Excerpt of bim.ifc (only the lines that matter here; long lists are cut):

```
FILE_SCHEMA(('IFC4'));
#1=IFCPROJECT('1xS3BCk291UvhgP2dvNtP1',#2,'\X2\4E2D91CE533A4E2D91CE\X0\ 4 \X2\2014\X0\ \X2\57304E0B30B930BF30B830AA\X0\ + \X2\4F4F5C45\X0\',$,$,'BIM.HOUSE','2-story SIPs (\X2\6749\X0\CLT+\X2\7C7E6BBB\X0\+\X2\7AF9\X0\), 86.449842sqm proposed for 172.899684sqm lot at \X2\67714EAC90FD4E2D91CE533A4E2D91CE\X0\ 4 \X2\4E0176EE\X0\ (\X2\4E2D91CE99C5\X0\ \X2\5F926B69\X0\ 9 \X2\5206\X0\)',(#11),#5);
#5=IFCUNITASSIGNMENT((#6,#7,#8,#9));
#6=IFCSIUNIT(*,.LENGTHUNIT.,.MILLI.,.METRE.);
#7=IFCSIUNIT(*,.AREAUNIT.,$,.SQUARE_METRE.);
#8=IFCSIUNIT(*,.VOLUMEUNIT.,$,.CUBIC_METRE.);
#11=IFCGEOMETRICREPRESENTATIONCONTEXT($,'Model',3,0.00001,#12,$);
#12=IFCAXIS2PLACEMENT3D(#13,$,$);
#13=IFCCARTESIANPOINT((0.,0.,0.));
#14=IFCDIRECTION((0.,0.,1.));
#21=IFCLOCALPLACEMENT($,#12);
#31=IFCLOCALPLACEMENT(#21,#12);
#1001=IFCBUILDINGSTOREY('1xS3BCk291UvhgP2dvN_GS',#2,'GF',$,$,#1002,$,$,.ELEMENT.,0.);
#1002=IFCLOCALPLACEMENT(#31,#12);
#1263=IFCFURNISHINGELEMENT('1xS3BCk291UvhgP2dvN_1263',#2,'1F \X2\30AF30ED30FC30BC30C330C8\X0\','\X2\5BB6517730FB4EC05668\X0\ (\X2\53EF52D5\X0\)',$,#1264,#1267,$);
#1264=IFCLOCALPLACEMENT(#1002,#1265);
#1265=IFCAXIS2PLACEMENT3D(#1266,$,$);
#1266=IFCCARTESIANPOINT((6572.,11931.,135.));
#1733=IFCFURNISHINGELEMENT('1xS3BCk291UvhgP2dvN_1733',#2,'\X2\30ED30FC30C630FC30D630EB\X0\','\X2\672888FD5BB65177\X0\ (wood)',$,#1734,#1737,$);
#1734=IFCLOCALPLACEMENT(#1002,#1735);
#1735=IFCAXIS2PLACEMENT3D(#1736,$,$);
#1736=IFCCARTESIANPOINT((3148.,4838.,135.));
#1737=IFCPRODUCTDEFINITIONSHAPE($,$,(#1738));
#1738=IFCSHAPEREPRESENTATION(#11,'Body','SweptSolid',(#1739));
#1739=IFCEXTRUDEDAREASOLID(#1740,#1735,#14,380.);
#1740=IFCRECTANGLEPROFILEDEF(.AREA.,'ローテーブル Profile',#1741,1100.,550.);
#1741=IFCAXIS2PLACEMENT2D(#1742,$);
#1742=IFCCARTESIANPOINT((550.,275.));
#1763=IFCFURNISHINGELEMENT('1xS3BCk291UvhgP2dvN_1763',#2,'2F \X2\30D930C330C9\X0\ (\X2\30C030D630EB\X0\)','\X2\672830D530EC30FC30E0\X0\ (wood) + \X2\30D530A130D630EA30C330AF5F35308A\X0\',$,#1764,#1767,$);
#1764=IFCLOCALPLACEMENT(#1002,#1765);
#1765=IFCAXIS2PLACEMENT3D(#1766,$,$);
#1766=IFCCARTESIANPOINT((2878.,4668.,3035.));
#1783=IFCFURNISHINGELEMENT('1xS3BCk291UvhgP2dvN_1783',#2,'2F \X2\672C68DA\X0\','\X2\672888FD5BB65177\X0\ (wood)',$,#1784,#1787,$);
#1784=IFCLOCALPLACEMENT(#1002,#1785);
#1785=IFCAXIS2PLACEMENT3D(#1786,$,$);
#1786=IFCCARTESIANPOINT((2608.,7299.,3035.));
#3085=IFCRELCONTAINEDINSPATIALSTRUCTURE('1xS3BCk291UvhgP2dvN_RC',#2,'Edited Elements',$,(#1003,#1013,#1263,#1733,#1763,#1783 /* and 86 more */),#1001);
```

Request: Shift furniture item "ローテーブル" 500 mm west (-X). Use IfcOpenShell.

```python
import ifcopenshell
import ifcopenshell.api.geometry
import ifcopenshell.util.placement

model = ifcopenshell.open("bim.ifc")

item = model.by_guid("1xS3BCk291UvhgP2dvN_1733")
matrix = ifcopenshell.util.placement.get_local_placement(item.ObjectPlacement)
matrix[0, 3] -= 500.0
ifcopenshell.api.geometry.edit_object_placement(model, product=item, matrix=matrix, is_si=False)

print(ifcopenshell.util.placement.get_local_placement(item.ObjectPlacement).round(3) + 0.0)

model.write("bim_edited.ifc")
```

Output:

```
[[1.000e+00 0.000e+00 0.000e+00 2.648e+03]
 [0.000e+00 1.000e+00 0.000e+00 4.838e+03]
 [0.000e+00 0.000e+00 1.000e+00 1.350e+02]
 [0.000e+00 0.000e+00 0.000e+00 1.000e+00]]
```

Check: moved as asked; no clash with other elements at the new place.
